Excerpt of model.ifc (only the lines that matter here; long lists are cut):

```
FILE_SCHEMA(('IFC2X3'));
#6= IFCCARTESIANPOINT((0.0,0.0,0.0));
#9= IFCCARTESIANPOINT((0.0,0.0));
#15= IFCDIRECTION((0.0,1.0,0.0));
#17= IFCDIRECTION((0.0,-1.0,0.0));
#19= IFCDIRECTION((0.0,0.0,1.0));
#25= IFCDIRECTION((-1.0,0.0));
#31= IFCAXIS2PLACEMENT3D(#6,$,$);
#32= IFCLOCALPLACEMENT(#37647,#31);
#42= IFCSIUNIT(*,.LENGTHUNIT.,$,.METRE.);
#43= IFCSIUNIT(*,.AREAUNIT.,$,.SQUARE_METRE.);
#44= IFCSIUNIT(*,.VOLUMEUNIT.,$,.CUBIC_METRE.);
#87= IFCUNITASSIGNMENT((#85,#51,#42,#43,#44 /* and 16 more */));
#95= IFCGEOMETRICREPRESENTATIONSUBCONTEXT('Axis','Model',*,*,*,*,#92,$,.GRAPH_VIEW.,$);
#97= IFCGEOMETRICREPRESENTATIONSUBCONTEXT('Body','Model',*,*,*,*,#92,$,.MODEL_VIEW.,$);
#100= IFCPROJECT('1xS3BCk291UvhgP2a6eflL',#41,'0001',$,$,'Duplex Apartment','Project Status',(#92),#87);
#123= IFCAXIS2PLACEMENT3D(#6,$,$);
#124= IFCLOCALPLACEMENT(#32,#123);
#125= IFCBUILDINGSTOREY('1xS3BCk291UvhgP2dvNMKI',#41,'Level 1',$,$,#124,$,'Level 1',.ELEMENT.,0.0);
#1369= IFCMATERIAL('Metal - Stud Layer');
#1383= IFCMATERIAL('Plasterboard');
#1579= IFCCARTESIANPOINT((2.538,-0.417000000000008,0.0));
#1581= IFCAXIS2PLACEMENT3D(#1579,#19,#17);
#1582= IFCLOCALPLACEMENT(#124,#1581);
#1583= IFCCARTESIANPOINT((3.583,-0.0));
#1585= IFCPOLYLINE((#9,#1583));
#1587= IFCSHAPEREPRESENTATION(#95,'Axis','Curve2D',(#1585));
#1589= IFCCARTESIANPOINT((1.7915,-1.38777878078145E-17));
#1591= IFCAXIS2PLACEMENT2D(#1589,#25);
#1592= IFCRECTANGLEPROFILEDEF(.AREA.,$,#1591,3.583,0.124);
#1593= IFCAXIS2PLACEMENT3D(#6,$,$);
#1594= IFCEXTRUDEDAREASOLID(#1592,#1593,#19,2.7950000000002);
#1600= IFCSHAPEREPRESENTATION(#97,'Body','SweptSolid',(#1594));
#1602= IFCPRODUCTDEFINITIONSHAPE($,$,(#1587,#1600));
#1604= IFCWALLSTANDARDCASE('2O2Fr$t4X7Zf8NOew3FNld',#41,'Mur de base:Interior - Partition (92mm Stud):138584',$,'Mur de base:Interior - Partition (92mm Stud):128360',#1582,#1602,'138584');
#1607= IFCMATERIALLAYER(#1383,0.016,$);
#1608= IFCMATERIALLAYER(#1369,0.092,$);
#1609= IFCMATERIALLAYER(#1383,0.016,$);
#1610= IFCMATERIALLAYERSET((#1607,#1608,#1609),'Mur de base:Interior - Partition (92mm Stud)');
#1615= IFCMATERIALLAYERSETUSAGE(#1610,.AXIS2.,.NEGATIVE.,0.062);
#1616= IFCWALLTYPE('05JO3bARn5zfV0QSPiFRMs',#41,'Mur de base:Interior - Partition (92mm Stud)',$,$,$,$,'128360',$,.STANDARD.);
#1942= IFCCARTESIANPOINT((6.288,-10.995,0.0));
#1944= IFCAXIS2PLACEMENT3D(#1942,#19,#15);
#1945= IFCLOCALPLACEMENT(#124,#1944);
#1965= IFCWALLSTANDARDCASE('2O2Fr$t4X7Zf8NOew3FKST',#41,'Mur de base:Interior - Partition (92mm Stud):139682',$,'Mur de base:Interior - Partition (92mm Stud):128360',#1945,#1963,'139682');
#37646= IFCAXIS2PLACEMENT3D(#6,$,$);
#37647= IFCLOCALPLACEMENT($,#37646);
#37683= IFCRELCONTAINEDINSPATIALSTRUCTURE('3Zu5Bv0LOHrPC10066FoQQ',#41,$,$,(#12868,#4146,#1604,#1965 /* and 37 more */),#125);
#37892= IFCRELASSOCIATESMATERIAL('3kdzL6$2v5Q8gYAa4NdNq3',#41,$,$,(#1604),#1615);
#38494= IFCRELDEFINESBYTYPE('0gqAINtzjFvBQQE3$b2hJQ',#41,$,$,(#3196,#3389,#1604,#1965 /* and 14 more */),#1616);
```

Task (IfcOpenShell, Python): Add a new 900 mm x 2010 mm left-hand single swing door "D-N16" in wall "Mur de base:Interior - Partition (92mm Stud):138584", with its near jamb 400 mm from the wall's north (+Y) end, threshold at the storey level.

```python
import numpy as np
import ifcopenshell
import ifcopenshell.api.feature
import ifcopenshell.api.geometry
import ifcopenshell.api.root
import ifcopenshell.api.spatial
import ifcopenshell.api.type
import ifcopenshell.geom
import ifcopenshell.util.element
import ifcopenshell.util.placement
import ifcopenshell.util.representation
import ifcopenshell.util.shape
import ifcopenshell.util.unit

model = ifcopenshell.open("model.ifc")
unit_scale = ifcopenshell.util.unit.calculate_unit_scale(model)
settings = ifcopenshell.geom.settings()


def volume(element):
    """Net volume in cubic metres, openings subtracted."""
    shape = ifcopenshell.geom.create_shape(settings, element)
    return ifcopenshell.util.shape.get_volume(shape.geometry)


wall = model.by_guid("2O2Fr$t4X7Zf8NOew3FNld")
storey = ifcopenshell.util.element.get_container(wall, ifc_class="IfcBuildingStorey")
context = ifcopenshell.util.representation.get_context(model, "Model", "Body", "MODEL_VIEW")
before = volume(wall)

width, height, from_end, sill = 0.9, 2.01, 0.4, 0.0  # metres

# The wall runs along its own X axis, and the end named is its -X end.
wall_shape = ifcopenshell.geom.create_shape(settings, wall)
x, y, z = ifcopenshell.util.shape.get_vertices(wall_shape.geometry).T
start = x.min() + from_end
face, thickness = float(y.min()), float(y.max() - y.min())
wall_matrix = ifcopenshell.util.placement.get_local_placement(wall.ObjectPlacement)
level = ifcopenshell.util.placement.get_local_placement(storey.ObjectPlacement)[2, 3]


def in_wall(x, y):
    """Placement at x, y metres in the wall's axes, at sill height."""
    matrix = wall_matrix.copy()
    matrix[:, 3] = wall_matrix @ np.array([x / unit_scale, y / unit_scale, 0.0, 1.0])
    matrix[2, 3] = level + sill / unit_scale
    return matrix


# Opening: a box that overshoots both wall faces by 50 mm.
opening = ifcopenshell.api.root.create_entity(model, ifc_class="IfcOpeningElement")
box = ifcopenshell.api.geometry.add_wall_representation(
    model, context=context, length=width, height=height, thickness=thickness + 0.1
)
ifcopenshell.api.geometry.assign_representation(model, product=opening, representation=box)
ifcopenshell.api.geometry.edit_object_placement(model, product=opening, matrix=in_wall(start, face - 0.05), is_si=False)
ifcopenshell.api.feature.add_feature(model, feature=opening, element=wall)

door = ifcopenshell.api.root.create_entity(model, ifc_class="IfcDoor", name="D-N16")
door.OverallWidth, door.OverallHeight = width / unit_scale, height / unit_scale
body = ifcopenshell.api.geometry.add_door_representation(
    model,
    context=context,
    overall_width=door.OverallWidth,
    overall_height=door.OverallHeight,
    operation_type="SINGLE_SWING_LEFT",
    lining_properties={"LiningDepth": thickness / unit_scale, "ThresholdDepth": thickness / unit_scale},
)
ifcopenshell.api.geometry.assign_representation(model, product=door, representation=body)
ifcopenshell.api.spatial.assign_container(model, products=[door], relating_structure=storey)
fills = ifcopenshell.api.feature.add_filling(model, opening=opening, element=door)
fills.OwnerHistory = door.OwnerHistory  # required in IFC2X3

# IFC2X3 keeps the operation on the door style.
style = ifcopenshell.api.root.create_entity(model, ifc_class="IfcDoorStyle", name="D-N16")
style.OperationType, style.ConstructionType = "SINGLE_SWING_LEFT", "NOTDEFINED"
style.ParameterTakesPrecedence = style.Sizeable = False
ifcopenshell.api.type.assign_type(model, related_objects=[door], relating_type=style)

# The lining spans the wall, so the door starts at the wall face.
ifcopenshell.api.geometry.edit_object_placement(model, product=door, matrix=in_wall(start, face), is_si=False)

after = volume(wall)

print(f"wall volume {before:.3f} -> {after:.3f} m3")

model.write("model_updated.ifc")
```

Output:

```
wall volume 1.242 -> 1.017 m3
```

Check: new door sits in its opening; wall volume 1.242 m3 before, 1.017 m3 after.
